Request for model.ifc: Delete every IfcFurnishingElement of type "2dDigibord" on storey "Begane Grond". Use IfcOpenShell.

First a look at what the model holds.

```python
import ifcopenshell
import ifcopenshell.util.element

model = ifcopenshell.open("model.ifc")
print(model.schema)
storey = next(s for s in model.by_type("IfcBuildingStorey") if s.Name == "Begane Grond")
furniture = [e for e in ifcopenshell.util.element.get_decomposition(storey) if e.is_a("IfcFurnishingElement")]
seen = {}
for e in furniture:
    element_type = ifcopenshell.util.element.get_type(e)
    name = element_type.Name if element_type not in (None, e) else None
    seen[name] = seen.get(name, 0) + 1
for name, count in sorted(seen.items(), key=str):
    print(count, "x", name)
```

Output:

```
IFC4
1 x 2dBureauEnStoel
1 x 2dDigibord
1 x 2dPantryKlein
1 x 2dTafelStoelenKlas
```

```python
import ifcopenshell
import ifcopenshell.api.root
import ifcopenshell.util.element

model = ifcopenshell.open("model.ifc")

storey = next(s for s in model.by_type("IfcBuildingStorey") if s.Name == "Begane Grond")
furniture = [e for e in ifcopenshell.util.element.get_decomposition(storey) if e.is_a("IfcFurnishingElement")]
targets = [e for e in furniture if (t := ifcopenshell.util.element.get_type(e)) not in (None, e) and t.Name == "2dDigibord"]

for e in targets:
    ifcopenshell.api.root.remove_product(model, product=e)
print(len(targets), "removed")

model.write("model_v2.ifc")
```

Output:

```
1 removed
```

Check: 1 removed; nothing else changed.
